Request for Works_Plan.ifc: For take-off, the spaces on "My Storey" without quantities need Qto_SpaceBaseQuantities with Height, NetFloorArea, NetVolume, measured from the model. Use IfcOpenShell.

First a look at what the model holds.

```python
import ifcopenshell
import ifcopenshell.util.element
import ifcopenshell.util.unit

model = ifcopenshell.open("Works_Plan.ifc")
print(model.schema)
for unit_type in ("LENGTHUNIT", "AREAUNIT", "VOLUMEUNIT"):
    print(unit_type, ifcopenshell.util.unit.calculate_unit_scale(model, unit_type))
storey = next(s for s in model.by_type("IfcBuildingStorey") if s.Name == "My Storey")
spaces = [e for e in ifcopenshell.util.element.get_decomposition(storey) if e.is_a("IfcSpace")]
for e in sorted(spaces, key=lambda e: e.id()):
    print(e.id(), e.is_a(), e.Name, list(ifcopenshell.util.element.get_psets(e, qtos_only=True)), sep=" | ")
```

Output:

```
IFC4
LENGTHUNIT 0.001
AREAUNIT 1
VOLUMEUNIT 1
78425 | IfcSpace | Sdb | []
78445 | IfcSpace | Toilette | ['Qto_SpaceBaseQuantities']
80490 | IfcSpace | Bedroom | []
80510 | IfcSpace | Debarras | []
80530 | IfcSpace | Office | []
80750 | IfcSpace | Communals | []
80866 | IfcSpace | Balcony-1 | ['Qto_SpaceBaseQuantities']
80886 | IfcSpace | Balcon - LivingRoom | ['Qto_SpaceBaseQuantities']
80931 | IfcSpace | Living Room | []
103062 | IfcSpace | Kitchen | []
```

```python
import ifcopenshell
import ifcopenshell.api.pset
import ifcopenshell.geom
import ifcopenshell.util.element
import ifcopenshell.util.shape
import ifcopenshell.util.unit

model = ifcopenshell.open("Works_Plan.ifc")
unit_scale = ifcopenshell.util.unit.calculate_unit_scale(model)
area_scale = ifcopenshell.util.unit.calculate_unit_scale(model, "AREAUNIT")
volume_scale = ifcopenshell.util.unit.calculate_unit_scale(model, "VOLUMEUNIT")
settings = ifcopenshell.geom.settings()

storey = next(s for s in model.by_type("IfcBuildingStorey") if s.Name == "My Storey")
spaces = [e for e in ifcopenshell.util.element.get_decomposition(storey) if e.is_a("IfcSpace")]

for e in sorted(spaces, key=lambda e: e.id()):
    if ifcopenshell.util.element.get_psets(e, qtos_only=True, should_inherit=False):
        continue
    # Geometry comes back in metres, in the element's own axes.
    shape = ifcopenshell.geom.create_shape(settings, e)
    values = {
        "Height": ifcopenshell.util.shape.get_z(shape.geometry) / unit_scale,
        "NetFloorArea": ifcopenshell.util.shape.get_footprint_area(shape.geometry) / area_scale,
        "NetVolume": ifcopenshell.util.shape.get_volume(shape.geometry) / volume_scale,
    }
    qto = ifcopenshell.api.pset.add_qto(model, product=e, name="Qto_SpaceBaseQuantities")
    ifcopenshell.api.pset.edit_qto(model, qto=qto, properties=values)
    print(e.id(), {k: round(v, 3) for k, v in values.items()})

model.write("Works_Plan_rev.ifc")
```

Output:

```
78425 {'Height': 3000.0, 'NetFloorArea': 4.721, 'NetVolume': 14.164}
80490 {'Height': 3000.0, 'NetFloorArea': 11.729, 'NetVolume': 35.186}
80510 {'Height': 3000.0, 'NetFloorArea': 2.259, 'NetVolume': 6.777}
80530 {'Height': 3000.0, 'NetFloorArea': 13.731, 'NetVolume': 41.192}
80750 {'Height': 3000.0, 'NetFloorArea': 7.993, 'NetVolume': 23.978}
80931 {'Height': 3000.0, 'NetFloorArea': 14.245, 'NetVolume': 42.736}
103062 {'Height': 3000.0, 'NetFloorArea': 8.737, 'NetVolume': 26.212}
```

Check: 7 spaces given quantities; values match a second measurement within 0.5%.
